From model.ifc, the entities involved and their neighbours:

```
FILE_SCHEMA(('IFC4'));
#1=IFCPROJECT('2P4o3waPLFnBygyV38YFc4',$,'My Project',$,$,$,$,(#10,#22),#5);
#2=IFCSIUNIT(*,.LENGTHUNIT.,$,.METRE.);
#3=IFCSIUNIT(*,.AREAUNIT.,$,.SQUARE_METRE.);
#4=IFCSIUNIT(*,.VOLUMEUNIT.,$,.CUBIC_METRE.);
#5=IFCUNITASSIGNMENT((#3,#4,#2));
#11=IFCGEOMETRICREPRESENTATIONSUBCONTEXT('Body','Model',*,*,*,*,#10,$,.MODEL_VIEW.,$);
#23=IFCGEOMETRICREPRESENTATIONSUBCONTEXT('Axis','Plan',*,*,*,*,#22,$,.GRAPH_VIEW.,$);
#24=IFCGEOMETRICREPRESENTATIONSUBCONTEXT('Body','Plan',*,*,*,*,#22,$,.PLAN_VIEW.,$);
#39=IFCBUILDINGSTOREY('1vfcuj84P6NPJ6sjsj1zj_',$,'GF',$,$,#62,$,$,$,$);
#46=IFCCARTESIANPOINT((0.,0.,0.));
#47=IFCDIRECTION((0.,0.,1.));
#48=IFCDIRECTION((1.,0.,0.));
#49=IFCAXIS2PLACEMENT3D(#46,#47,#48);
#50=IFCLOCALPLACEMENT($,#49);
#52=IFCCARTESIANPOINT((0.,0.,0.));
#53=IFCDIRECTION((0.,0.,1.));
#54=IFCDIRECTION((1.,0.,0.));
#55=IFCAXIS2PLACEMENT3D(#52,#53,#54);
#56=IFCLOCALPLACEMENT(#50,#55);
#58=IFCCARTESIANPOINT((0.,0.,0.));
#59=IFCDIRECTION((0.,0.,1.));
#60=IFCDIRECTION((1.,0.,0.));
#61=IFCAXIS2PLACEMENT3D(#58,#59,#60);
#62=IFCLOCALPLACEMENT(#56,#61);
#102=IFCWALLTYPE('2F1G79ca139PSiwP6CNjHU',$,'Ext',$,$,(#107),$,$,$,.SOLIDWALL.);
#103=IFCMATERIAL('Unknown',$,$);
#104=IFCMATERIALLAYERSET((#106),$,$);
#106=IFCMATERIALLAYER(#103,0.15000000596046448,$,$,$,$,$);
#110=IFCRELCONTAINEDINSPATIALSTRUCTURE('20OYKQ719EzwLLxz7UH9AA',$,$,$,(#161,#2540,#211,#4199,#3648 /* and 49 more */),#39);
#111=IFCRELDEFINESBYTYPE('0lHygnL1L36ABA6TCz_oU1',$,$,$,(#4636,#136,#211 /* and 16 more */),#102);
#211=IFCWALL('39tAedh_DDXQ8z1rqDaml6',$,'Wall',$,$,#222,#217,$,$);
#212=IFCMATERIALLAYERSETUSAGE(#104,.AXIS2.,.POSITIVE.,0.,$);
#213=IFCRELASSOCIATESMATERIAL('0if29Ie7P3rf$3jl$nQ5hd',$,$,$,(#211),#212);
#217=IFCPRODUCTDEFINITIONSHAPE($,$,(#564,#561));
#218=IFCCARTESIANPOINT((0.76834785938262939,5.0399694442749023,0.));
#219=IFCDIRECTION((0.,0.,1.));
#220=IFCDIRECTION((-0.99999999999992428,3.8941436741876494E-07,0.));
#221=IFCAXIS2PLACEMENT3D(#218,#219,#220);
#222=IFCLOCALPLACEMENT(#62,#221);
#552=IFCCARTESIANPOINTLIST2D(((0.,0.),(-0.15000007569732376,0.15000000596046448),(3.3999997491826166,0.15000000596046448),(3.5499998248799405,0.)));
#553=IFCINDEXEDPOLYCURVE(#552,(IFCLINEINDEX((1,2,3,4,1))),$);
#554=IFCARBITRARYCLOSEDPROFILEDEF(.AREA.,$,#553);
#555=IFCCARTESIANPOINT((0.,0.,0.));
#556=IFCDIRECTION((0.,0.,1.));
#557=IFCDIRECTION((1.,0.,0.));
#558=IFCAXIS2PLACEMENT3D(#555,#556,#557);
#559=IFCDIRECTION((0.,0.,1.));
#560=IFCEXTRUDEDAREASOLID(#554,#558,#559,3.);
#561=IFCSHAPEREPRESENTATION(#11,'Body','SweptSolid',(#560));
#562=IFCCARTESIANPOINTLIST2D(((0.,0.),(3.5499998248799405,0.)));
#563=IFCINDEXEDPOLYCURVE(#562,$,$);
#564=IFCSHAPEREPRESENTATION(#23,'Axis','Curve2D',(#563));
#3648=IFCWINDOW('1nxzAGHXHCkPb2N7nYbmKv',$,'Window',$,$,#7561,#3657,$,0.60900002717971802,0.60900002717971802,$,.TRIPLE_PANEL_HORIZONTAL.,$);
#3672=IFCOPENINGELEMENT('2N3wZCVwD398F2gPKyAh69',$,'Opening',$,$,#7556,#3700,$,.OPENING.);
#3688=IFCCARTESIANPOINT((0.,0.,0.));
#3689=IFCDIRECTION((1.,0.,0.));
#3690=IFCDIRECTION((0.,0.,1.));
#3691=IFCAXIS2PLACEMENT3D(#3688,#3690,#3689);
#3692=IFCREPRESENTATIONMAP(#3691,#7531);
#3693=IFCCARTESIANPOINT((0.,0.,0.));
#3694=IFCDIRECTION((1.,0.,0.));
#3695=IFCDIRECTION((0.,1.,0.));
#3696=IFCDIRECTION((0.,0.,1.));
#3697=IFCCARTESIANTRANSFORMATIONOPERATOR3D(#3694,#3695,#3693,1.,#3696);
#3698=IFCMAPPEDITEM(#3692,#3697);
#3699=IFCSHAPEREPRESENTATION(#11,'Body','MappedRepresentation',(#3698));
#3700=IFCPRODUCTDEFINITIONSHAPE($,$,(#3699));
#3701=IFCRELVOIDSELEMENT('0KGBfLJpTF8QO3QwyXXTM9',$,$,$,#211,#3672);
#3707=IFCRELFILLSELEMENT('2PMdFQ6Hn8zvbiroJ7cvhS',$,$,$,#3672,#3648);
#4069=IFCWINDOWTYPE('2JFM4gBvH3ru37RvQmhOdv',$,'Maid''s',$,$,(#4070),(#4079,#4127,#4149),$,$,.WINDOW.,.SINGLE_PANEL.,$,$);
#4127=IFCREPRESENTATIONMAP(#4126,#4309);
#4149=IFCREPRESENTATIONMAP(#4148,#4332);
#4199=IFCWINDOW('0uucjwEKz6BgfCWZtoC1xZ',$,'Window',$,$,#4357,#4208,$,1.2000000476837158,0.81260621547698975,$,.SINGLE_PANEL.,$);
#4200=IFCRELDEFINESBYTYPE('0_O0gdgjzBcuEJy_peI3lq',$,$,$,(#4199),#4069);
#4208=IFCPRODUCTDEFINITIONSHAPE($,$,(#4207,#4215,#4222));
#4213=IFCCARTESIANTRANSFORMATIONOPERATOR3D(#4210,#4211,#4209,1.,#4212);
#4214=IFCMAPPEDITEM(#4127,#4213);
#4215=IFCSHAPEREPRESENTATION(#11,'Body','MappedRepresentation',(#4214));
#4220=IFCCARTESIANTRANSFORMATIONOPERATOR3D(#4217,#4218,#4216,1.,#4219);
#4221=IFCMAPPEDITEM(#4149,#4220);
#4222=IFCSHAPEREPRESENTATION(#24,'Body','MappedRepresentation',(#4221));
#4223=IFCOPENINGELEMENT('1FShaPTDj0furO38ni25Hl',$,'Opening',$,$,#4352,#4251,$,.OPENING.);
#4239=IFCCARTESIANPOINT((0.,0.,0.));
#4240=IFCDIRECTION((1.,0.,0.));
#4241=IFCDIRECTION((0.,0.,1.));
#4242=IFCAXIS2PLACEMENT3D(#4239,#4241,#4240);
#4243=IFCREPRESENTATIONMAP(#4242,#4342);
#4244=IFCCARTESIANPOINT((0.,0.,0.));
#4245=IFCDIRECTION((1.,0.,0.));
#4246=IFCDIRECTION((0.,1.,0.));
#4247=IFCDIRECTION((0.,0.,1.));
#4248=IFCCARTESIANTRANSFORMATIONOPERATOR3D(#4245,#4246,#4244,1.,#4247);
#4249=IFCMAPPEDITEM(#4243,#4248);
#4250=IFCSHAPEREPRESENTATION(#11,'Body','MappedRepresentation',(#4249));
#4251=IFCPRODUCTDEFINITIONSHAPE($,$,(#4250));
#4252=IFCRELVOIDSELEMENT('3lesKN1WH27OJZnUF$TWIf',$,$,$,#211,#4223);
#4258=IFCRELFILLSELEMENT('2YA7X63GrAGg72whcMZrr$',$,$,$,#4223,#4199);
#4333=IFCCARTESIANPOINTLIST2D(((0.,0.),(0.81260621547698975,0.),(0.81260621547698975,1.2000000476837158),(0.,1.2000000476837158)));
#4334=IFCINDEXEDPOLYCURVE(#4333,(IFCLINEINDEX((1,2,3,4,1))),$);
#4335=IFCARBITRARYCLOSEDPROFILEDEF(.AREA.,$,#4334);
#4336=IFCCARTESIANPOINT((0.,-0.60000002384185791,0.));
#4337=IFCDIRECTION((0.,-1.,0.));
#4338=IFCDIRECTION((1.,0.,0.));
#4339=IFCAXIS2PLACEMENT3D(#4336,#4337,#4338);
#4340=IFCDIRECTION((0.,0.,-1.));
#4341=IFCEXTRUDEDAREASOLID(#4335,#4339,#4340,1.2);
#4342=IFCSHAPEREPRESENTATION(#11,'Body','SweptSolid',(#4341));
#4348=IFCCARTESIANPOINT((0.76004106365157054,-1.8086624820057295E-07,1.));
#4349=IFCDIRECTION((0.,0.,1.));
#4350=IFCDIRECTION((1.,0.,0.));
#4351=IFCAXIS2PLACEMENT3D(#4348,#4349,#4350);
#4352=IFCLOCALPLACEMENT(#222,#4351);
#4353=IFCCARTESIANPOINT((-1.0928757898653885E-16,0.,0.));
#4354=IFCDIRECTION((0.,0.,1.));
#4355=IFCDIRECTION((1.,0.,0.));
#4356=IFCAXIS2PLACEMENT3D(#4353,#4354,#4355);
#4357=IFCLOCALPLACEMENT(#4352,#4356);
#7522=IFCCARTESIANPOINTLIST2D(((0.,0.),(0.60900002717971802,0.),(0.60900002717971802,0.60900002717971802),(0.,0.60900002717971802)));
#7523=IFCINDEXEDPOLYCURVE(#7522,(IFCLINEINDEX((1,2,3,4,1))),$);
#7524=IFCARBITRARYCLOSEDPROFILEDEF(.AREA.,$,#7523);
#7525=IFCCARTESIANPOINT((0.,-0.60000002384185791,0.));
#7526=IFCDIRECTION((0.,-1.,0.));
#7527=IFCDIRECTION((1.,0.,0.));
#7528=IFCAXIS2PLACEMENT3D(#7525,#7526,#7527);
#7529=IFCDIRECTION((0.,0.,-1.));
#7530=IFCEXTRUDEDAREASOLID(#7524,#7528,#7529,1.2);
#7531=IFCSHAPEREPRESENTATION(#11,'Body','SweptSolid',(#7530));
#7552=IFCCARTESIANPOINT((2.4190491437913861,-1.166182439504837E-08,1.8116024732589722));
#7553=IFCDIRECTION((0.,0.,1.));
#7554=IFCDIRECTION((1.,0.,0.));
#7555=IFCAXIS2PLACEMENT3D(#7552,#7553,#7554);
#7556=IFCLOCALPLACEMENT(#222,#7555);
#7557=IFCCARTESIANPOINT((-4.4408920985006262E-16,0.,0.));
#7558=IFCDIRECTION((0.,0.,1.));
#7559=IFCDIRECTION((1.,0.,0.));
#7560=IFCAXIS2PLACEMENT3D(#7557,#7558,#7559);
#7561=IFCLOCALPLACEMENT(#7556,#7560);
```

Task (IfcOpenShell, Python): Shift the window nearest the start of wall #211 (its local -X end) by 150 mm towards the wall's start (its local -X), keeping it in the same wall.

```python
import ifcopenshell
import ifcopenshell.api.geometry
import ifcopenshell.util.placement

model = ifcopenshell.open("model.ifc")

window = model.by_guid("0uucjwEKz6BgfCWZtoC1xZ")
opening = window.FillsVoids[0].RelatingOpeningElement
wall = opening.VoidsElements[0].RelatingBuildingElement

wall_matrix = ifcopenshell.util.placement.get_local_placement(wall.ObjectPlacement)
shift = wall_matrix[:3, 0] * -0.15
before = ifcopenshell.util.placement.get_local_placement(window.ObjectPlacement)[:3, 3].copy()

# The window is placed relative to its opening, so it follows when the opening moves.
matrix = ifcopenshell.util.placement.get_local_placement(opening.ObjectPlacement)
matrix[:3, 3] += shift
ifcopenshell.api.geometry.edit_object_placement(
    model, product=opening, matrix=matrix, is_si=False, should_transform_children=True
)

after = ifcopenshell.util.placement.get_local_placement(window.ObjectPlacement)[:3, 3]
print("window moved by", (after - before).round(3) + 0.0)

model.write("model_rev.ifc")
```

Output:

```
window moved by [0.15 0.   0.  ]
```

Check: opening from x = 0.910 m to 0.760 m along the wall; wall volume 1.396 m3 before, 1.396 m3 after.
